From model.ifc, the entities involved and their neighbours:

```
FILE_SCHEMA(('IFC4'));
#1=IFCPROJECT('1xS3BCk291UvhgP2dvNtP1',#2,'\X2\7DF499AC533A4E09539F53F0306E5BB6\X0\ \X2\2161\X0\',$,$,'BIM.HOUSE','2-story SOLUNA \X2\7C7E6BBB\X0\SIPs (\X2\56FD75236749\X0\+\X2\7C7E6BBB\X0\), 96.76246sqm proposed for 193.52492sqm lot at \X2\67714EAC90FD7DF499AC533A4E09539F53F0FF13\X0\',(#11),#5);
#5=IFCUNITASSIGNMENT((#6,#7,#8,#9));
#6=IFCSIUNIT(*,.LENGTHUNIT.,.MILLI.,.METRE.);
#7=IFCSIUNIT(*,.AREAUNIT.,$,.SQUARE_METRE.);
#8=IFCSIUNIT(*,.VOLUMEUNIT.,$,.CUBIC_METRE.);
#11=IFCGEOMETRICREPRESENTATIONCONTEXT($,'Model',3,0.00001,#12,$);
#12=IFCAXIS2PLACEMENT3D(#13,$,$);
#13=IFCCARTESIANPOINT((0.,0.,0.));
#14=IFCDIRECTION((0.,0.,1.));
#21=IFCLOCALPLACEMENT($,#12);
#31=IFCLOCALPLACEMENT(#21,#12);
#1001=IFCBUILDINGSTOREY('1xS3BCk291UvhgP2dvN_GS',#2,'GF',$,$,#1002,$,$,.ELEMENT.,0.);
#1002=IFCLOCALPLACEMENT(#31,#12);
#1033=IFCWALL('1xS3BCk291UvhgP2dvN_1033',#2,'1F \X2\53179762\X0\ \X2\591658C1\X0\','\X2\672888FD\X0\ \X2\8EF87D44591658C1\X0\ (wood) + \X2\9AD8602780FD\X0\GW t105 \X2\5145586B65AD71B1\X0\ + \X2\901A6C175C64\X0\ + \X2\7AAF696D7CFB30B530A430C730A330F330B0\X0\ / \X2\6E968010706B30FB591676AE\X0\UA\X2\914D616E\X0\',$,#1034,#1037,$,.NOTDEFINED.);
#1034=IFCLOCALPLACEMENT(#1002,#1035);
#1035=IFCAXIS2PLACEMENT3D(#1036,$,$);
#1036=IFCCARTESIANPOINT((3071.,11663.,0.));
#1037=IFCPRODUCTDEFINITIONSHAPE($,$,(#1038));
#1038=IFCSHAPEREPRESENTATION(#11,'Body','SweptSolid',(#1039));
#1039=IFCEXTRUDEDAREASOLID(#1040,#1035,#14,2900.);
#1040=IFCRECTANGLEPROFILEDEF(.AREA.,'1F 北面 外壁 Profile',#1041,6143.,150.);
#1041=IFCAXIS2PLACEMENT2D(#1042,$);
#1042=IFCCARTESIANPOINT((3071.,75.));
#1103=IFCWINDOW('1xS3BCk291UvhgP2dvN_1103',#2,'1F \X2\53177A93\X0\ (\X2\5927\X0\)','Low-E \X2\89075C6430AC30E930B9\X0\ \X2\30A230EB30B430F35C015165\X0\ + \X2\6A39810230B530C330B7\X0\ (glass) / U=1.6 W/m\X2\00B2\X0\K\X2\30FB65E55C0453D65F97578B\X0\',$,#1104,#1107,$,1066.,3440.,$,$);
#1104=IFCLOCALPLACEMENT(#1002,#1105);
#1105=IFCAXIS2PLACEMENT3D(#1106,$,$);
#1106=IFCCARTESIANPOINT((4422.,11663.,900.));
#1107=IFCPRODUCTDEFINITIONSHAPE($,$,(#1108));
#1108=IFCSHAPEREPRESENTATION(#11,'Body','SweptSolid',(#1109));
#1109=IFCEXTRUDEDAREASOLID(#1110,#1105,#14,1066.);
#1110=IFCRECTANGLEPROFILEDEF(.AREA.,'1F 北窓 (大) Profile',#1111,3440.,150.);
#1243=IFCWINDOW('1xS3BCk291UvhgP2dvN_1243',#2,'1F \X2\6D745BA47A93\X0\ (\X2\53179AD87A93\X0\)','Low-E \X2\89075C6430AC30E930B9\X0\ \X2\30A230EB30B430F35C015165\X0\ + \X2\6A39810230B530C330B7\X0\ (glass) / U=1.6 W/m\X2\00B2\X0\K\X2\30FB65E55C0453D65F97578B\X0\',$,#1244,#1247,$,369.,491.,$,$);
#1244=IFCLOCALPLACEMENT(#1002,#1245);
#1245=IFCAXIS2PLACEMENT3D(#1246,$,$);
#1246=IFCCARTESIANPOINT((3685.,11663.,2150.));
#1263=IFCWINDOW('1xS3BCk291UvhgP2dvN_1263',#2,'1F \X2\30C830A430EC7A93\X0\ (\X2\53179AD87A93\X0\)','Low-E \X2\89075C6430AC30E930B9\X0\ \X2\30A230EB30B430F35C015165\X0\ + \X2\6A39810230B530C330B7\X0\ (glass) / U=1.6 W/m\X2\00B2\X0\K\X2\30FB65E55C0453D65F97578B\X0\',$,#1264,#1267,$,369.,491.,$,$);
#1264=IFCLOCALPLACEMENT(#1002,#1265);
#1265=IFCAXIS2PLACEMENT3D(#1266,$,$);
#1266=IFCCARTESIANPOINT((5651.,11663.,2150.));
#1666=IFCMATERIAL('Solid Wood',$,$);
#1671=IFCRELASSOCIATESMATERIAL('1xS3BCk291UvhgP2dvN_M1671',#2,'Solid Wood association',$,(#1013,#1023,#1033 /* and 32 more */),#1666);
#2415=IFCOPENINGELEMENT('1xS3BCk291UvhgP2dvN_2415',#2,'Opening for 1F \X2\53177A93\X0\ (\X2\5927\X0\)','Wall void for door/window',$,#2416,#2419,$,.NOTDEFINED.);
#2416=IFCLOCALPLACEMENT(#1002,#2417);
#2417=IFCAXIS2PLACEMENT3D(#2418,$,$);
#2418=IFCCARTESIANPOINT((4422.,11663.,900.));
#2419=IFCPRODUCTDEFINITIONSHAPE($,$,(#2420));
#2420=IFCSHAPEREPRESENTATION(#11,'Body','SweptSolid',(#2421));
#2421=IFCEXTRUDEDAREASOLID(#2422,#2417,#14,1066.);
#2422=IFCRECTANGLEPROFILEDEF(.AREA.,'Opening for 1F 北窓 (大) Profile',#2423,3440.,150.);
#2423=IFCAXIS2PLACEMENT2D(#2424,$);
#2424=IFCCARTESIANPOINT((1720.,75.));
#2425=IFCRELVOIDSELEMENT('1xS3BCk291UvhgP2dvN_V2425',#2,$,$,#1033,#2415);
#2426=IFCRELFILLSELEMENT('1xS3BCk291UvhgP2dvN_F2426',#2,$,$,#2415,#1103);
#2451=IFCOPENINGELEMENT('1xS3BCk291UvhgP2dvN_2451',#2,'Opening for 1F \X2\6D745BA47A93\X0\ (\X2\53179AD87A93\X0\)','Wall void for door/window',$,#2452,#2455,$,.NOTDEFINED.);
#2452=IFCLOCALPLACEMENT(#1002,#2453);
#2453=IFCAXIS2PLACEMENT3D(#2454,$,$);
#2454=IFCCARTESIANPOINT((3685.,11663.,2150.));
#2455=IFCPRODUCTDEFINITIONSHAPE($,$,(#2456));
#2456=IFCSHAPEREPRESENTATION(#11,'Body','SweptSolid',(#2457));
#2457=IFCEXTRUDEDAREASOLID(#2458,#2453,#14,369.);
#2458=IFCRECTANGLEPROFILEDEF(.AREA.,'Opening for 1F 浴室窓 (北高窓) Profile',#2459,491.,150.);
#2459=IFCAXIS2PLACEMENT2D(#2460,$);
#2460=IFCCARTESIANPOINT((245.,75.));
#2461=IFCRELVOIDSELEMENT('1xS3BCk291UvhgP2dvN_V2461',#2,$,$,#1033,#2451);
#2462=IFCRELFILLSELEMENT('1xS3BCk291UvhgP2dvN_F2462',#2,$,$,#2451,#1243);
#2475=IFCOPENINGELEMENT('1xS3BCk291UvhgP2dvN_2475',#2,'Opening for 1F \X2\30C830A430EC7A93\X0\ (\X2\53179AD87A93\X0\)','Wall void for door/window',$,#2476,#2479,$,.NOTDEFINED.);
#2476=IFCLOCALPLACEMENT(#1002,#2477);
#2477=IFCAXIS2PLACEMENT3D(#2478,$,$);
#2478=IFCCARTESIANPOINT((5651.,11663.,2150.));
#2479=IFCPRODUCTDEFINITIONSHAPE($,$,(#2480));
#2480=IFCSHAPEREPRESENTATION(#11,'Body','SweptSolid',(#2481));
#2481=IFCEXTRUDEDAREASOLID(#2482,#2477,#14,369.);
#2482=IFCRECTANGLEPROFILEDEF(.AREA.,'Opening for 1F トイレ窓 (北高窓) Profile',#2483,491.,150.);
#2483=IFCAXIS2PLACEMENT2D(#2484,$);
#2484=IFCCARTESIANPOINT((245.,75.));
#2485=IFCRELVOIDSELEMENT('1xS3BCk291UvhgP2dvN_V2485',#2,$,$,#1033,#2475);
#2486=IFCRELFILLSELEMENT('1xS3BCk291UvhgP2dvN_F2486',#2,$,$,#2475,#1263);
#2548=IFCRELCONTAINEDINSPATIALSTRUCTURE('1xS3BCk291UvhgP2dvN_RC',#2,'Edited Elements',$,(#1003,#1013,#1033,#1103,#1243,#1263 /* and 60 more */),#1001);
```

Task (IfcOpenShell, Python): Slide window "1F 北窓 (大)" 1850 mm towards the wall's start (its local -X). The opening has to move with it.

```python
import ifcopenshell
import ifcopenshell.api.geometry
import ifcopenshell.util.placement
import ifcopenshell.util.unit

model = ifcopenshell.open("model.ifc")
unit_scale = ifcopenshell.util.unit.calculate_unit_scale(model)

window = model.by_id(1103)
opening = window.FillsVoids[0].RelatingOpeningElement
wall = opening.VoidsElements[0].RelatingBuildingElement

wall_matrix = ifcopenshell.util.placement.get_local_placement(wall.ObjectPlacement)
shift = wall_matrix[:3, 0] * -1.85 / unit_scale
before = ifcopenshell.util.placement.get_local_placement(window.ObjectPlacement)[:3, 3].copy()

# The window is not placed relative to its opening, so move both.
for product in (opening, window):
    matrix = ifcopenshell.util.placement.get_local_placement(product.ObjectPlacement)
    matrix[:3, 3] += shift
    ifcopenshell.api.geometry.edit_object_placement(model, product=product, matrix=matrix, is_si=False)

after = ifcopenshell.util.placement.get_local_placement(window.ObjectPlacement)[:3, 3]
print("window moved by", (after - before).round(3) + 0.0)

model.write("model_edited.ifc")
```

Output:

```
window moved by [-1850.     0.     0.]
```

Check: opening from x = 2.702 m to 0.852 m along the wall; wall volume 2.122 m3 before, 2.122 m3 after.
